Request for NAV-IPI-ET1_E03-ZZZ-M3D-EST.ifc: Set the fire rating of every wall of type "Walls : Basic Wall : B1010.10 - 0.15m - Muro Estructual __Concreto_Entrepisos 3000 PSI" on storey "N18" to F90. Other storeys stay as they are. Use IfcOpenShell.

First a look at what the model holds.

```python
import ifcopenshell
import ifcopenshell.util.element

model = ifcopenshell.open("NAV-IPI-ET1_E03-ZZZ-M3D-EST.ifc")
print(model.schema)
storey = next(s for s in model.by_type("IfcBuildingStorey") if s.Name == "N18")
walls = [e for e in ifcopenshell.util.element.get_decomposition(storey) if e.is_a("IfcWall")]
seen = {}
for e in walls:
    element_type = ifcopenshell.util.element.get_type(e)
    key = (element_type.Name if element_type != e and element_type else None, ifcopenshell.util.element.get_pset(e, "Pset_WallCommon", "FireRating"))
    seen[key] = seen.get(key, 0) + 1
for (name, value), count in sorted(seen.items(), key=str):
    print(count, "x", name, "|", value)
```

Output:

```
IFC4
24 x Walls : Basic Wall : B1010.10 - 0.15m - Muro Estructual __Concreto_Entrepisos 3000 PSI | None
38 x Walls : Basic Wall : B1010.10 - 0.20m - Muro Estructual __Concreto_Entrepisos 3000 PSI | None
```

```python
import ifcopenshell
import ifcopenshell.api.pset
import ifcopenshell.util.element

model = ifcopenshell.open("NAV-IPI-ET1_E03-ZZZ-M3D-EST.ifc")

storey = next(s for s in model.by_type("IfcBuildingStorey") if s.Name == "N18")
walls = [e for e in ifcopenshell.util.element.get_decomposition(storey) if e.is_a("IfcWall")]

count = 0
for e in walls:
    element_type = ifcopenshell.util.element.get_type(e)
    if element_type in (None, e) or element_type.Name != "Walls : Basic Wall : B1010.10 - 0.15m - Muro Estructual __Concreto_Entrepisos 3000 PSI":
        continue
    # add_pset returns the element's existing set when there is one.
    pset = ifcopenshell.api.pset.add_pset(model, product=e, name="Pset_WallCommon")
    ifcopenshell.api.pset.edit_pset(model, pset=pset, properties={"FireRating": "F90"})
    count += 1

print(count, "walls updated")

model.write("NAV-IPI-ET1_E03-ZZZ-M3D-EST-out.ifc")
```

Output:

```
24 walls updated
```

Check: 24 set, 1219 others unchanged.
